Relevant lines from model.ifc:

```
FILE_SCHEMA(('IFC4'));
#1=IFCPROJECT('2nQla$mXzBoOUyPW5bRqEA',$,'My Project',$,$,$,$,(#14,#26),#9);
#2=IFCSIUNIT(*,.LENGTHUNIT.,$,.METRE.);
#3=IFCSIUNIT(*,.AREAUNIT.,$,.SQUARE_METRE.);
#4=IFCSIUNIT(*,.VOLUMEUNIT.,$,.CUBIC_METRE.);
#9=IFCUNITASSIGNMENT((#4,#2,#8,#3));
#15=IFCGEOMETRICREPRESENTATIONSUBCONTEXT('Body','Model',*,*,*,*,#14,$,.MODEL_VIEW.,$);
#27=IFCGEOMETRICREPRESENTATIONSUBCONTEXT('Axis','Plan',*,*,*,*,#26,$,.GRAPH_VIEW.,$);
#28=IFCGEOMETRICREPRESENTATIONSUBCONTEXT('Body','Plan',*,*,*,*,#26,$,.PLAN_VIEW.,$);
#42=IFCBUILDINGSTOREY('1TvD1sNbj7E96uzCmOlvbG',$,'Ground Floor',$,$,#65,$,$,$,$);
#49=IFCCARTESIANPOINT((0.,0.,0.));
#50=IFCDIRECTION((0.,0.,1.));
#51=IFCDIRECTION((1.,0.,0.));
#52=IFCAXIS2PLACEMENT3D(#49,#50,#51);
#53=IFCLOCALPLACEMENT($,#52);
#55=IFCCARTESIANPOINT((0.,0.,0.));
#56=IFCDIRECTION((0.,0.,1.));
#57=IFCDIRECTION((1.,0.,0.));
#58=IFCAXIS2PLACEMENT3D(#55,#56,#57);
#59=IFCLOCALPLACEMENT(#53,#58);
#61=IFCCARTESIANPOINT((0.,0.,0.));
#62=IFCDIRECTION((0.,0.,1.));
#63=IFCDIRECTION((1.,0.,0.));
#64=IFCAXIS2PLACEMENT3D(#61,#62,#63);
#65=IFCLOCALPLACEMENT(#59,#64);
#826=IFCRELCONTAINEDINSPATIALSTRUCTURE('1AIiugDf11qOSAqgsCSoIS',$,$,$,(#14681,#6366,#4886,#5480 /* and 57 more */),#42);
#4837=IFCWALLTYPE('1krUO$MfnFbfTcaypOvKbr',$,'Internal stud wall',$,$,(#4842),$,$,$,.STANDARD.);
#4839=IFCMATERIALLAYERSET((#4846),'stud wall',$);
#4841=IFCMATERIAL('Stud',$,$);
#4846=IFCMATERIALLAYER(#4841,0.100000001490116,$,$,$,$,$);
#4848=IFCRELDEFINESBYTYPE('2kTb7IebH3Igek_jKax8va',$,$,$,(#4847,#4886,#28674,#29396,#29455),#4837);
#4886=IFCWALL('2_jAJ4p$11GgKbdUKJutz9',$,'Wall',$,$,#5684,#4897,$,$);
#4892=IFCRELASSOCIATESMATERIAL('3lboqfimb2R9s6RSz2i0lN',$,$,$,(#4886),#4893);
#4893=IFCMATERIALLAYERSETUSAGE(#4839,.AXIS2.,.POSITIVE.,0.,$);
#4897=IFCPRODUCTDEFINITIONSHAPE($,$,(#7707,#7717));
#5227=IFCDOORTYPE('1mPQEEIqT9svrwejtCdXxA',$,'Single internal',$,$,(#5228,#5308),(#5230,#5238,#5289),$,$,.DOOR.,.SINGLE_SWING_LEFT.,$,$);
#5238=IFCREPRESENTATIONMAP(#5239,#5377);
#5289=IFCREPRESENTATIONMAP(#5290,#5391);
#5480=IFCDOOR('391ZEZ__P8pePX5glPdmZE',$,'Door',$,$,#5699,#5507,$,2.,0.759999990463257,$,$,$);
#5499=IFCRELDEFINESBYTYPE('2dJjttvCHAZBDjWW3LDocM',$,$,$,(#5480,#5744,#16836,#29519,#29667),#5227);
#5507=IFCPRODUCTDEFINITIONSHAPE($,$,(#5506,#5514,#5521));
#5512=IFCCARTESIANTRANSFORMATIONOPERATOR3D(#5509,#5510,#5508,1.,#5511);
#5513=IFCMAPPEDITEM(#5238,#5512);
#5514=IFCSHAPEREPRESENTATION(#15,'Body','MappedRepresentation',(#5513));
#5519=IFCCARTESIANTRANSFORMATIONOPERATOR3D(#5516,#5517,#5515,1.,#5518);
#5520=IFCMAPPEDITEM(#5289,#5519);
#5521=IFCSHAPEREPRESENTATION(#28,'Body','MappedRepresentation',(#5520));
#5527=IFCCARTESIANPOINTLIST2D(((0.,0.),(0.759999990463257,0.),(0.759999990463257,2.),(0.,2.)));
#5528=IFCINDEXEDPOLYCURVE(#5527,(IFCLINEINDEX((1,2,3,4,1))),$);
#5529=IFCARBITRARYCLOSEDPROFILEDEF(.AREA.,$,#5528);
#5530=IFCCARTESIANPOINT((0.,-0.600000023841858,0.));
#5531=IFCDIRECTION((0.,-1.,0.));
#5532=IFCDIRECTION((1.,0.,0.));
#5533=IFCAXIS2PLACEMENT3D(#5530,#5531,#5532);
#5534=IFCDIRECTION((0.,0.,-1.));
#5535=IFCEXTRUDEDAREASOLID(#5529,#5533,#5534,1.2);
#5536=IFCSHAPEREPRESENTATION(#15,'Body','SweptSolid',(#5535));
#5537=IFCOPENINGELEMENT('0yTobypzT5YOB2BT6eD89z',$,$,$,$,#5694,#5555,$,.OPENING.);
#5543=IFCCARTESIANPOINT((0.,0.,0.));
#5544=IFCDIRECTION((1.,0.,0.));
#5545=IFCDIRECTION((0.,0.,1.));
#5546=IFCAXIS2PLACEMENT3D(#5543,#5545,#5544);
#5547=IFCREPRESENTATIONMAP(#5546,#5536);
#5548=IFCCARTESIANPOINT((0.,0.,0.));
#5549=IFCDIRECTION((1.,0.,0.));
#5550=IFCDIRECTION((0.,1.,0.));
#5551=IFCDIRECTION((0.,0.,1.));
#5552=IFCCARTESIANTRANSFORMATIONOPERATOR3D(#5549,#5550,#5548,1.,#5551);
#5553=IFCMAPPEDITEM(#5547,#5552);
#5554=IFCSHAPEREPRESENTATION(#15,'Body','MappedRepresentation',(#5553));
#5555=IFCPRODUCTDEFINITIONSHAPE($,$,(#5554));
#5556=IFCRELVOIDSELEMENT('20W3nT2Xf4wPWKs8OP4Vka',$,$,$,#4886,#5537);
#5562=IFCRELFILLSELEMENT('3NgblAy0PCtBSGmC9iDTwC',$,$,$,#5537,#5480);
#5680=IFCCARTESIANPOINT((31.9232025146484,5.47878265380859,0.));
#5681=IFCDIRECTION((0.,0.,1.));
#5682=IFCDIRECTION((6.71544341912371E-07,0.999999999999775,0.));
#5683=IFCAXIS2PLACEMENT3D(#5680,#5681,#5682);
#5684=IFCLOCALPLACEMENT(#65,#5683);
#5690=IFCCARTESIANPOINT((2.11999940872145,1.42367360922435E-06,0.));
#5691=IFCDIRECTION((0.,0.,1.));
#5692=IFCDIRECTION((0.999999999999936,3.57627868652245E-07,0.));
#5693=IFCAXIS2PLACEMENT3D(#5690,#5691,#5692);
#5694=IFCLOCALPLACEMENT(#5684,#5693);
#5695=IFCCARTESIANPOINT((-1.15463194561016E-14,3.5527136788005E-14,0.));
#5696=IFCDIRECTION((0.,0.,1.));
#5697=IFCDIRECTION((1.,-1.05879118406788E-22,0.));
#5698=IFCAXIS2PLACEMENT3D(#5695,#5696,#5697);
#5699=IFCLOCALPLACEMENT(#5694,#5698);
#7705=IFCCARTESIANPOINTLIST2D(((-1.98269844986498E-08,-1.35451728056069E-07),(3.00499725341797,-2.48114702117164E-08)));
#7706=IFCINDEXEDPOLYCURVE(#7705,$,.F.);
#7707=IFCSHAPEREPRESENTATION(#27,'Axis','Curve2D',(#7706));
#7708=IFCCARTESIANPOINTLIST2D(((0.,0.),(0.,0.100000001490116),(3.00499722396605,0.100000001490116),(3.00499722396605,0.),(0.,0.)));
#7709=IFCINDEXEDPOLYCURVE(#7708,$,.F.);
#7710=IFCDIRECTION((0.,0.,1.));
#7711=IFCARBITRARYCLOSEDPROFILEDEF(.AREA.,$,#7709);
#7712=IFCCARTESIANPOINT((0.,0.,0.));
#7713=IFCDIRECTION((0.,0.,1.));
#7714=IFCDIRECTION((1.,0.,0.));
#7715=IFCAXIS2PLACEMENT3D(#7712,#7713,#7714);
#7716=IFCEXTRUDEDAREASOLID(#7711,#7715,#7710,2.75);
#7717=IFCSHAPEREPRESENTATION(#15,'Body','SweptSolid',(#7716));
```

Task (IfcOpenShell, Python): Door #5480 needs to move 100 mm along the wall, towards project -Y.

```python
import ifcopenshell
import ifcopenshell.api.geometry
import ifcopenshell.util.placement

model = ifcopenshell.open("model.ifc")

door = model.by_guid("391ZEZ__P8pePX5glPdmZE")
opening = door.FillsVoids[0].RelatingOpeningElement
wall = opening.VoidsElements[0].RelatingBuildingElement

wall_matrix = ifcopenshell.util.placement.get_local_placement(wall.ObjectPlacement)
shift = wall_matrix[:3, 0] * -0.1
before = ifcopenshell.util.placement.get_local_placement(door.ObjectPlacement)[:3, 3].copy()

# The door is placed relative to its opening, so it follows when the opening moves.
matrix = ifcopenshell.util.placement.get_local_placement(opening.ObjectPlacement)
matrix[:3, 3] += shift
ifcopenshell.api.geometry.edit_object_placement(
    model, product=opening, matrix=matrix, is_si=False, should_transform_children=True
)

after = ifcopenshell.util.placement.get_local_placement(door.ObjectPlacement)[:3, 3]
print("door moved by", (after - before).round(3) + 0.0)

model.write("model_v2.ifc")
```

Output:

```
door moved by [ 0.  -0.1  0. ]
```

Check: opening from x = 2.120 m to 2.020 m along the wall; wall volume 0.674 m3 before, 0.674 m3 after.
